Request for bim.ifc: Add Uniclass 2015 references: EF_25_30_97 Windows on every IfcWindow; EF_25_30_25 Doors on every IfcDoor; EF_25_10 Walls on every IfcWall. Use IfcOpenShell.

First a look at what the model holds.

```python
import ifcopenshell

model = ifcopenshell.open("bim.ifc")
print(model.schema)
print("classifications:", [c.Name for c in model.by_type("IfcClassification")])
for ifc_class in ("IfcDoor", "IfcRoof", "IfcStair", "IfcWall", "IfcWindow"):
    print(ifc_class, len(model.by_type(ifc_class)))
```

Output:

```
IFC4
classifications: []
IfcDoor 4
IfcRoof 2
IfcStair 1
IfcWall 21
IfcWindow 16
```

```python
import ifcopenshell
import ifcopenshell.api.classification

model = ifcopenshell.open("bim.ifc")

system = ifcopenshell.api.classification.add_classification(model, classification="Uniclass 2015")

codes = {
    "IfcWindow": ("EF_25_30_97", "Windows"),
    "IfcDoor": ("EF_25_30_25", "Doors"),
    "IfcWall": ("EF_25_10", "Walls"),
}
for ifc_class, (code, name) in codes.items():
    products = model.by_type(ifc_class)
    ifcopenshell.api.classification.add_reference(
        model, products=products, classification=system, identification=code, name=name
    )
    print(code, len(products))

model.write("bim_edited.ifc")
```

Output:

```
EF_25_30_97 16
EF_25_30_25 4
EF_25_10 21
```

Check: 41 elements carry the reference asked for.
